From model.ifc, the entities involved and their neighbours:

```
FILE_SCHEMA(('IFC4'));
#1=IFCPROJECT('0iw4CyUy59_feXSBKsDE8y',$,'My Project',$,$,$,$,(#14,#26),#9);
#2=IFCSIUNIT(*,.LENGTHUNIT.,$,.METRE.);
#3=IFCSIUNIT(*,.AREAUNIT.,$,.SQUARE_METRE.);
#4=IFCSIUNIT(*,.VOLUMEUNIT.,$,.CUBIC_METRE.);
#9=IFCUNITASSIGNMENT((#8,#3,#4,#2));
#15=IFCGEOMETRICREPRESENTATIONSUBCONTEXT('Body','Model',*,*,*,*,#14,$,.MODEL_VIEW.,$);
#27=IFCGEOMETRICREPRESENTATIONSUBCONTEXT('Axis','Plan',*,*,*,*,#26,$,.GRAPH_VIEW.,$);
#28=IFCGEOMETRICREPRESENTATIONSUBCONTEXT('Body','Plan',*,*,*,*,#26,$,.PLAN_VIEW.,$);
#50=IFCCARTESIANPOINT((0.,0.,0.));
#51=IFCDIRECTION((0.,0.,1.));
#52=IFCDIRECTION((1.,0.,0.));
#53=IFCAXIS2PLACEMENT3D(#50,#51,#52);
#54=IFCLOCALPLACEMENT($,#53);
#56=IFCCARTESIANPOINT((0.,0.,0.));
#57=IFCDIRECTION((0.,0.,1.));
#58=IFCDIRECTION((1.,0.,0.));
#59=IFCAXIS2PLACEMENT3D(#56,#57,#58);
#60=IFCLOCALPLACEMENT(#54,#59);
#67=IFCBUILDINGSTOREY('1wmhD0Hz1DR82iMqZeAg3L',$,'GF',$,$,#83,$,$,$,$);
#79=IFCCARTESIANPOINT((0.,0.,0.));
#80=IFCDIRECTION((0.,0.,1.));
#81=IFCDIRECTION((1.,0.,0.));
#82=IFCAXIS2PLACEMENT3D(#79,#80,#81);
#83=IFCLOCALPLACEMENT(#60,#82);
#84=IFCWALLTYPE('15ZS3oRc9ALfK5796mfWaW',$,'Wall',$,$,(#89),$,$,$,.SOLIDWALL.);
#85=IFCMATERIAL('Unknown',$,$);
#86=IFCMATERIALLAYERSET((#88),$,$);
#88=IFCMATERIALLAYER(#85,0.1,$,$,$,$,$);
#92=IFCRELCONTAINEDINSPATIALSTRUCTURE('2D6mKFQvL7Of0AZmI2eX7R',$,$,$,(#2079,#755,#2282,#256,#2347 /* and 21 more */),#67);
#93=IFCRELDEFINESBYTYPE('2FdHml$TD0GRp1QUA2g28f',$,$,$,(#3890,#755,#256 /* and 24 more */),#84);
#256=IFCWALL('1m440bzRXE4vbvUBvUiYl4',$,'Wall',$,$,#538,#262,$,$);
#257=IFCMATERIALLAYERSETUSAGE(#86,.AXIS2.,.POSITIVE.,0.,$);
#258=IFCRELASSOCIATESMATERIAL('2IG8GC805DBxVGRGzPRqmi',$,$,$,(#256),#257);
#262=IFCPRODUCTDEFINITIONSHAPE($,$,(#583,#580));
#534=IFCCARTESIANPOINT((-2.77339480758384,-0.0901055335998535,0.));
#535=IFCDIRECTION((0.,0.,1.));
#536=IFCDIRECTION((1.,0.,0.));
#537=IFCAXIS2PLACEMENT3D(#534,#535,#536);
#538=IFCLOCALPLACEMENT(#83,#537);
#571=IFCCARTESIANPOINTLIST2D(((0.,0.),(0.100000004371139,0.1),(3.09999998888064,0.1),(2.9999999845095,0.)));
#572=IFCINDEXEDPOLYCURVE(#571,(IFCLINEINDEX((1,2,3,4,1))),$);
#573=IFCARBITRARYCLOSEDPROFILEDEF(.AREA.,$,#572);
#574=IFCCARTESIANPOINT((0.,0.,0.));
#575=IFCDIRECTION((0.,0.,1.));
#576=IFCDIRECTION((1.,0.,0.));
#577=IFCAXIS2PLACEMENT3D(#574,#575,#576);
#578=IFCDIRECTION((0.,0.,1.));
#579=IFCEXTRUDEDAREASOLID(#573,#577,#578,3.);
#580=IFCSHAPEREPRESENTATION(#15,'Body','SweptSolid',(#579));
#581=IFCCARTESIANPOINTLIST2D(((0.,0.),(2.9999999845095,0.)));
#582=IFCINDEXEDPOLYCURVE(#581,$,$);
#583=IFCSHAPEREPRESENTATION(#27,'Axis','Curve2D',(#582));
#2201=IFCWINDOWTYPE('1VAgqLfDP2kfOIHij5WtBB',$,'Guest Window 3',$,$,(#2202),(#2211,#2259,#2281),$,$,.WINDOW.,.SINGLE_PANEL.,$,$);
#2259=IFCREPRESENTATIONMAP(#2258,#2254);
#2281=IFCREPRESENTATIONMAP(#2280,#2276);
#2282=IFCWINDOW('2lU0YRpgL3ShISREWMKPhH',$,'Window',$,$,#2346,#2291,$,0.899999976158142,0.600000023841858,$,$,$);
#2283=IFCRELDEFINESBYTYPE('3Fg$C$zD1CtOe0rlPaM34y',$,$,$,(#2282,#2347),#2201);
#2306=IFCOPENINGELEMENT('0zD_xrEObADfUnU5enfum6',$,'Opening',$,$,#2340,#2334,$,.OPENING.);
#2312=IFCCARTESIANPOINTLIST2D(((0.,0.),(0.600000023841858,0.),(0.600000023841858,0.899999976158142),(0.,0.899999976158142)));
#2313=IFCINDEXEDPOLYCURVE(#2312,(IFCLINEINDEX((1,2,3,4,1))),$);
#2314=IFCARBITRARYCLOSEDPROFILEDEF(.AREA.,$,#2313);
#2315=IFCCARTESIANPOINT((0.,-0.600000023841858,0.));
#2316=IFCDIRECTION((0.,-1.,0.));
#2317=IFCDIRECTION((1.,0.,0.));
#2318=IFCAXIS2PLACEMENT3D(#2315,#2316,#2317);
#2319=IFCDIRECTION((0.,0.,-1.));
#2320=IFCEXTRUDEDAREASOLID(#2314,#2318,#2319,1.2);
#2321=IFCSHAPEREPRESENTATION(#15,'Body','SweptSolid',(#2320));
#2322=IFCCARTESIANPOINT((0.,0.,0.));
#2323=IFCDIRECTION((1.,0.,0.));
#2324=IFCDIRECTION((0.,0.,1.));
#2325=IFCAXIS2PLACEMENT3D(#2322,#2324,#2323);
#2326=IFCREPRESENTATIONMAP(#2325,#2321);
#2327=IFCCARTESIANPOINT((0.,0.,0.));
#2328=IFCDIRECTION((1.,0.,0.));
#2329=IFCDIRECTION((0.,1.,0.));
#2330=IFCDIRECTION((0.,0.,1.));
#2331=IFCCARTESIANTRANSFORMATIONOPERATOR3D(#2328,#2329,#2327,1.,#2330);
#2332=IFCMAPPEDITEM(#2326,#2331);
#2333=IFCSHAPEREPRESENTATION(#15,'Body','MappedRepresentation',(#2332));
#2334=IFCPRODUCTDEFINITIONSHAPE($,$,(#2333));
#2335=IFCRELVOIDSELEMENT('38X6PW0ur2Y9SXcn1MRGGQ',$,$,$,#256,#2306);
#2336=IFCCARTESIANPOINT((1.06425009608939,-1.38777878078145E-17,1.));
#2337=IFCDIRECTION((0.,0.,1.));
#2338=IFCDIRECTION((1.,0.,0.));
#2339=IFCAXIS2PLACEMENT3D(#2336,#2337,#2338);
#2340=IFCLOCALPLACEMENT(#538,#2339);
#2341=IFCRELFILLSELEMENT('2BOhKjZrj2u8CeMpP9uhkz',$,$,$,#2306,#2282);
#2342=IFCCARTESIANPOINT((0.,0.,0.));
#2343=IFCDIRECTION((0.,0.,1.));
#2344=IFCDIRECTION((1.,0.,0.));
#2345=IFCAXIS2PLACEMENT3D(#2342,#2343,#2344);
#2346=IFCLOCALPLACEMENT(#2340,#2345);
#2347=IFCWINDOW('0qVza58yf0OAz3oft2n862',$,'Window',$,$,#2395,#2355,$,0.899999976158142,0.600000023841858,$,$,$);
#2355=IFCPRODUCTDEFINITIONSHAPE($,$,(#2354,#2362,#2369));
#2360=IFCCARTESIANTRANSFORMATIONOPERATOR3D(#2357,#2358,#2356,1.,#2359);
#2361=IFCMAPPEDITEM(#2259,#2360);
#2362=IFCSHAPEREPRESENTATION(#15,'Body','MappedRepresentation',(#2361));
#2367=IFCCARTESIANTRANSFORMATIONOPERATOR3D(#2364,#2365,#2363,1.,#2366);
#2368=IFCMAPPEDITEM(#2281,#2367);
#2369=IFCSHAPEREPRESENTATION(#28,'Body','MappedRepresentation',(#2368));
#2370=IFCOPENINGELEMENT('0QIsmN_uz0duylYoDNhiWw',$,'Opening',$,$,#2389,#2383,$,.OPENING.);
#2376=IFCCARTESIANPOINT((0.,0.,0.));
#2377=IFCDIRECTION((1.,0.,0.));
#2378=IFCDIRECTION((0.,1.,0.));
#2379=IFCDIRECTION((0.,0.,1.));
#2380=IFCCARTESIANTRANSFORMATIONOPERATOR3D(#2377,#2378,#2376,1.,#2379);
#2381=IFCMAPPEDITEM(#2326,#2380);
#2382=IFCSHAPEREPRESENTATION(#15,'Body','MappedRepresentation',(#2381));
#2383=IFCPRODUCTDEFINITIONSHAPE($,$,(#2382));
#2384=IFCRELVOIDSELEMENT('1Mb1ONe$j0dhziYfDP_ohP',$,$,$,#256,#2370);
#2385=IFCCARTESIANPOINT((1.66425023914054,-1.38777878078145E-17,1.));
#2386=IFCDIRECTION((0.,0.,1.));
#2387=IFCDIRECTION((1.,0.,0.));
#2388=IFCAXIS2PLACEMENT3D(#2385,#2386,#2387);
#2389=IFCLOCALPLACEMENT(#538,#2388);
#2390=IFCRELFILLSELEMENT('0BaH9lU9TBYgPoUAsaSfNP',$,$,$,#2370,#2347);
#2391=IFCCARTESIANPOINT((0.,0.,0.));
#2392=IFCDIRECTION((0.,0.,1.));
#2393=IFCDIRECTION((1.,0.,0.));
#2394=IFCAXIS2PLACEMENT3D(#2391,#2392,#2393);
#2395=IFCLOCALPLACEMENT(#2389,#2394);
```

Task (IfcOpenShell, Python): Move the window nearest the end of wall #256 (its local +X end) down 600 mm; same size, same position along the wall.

```python
import numpy as np
import ifcopenshell
import ifcopenshell.api.geometry
import ifcopenshell.util.placement
import ifcopenshell.util.unit

model = ifcopenshell.open("model.ifc")
unit_scale = ifcopenshell.util.unit.calculate_unit_scale(model)

window = model.by_guid("0qVza58yf0OAz3oft2n862")
opening = window.FillsVoids[0].RelatingOpeningElement
dz = -0.6 / unit_scale

shift = np.array([0.0, 0.0, dz])
# The window is placed relative to its opening, so it follows when the opening moves.
matrix = ifcopenshell.util.placement.get_local_placement(opening.ObjectPlacement)
matrix[:3, 3] += shift
ifcopenshell.api.geometry.edit_object_placement(
    model, product=opening, matrix=matrix, is_si=False, should_transform_children=True
)

print(f"moved by {dz * unit_scale:+.3f} m")

model.write("model_edited.ifc")
```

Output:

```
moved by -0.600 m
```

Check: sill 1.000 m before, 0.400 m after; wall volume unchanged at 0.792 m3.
